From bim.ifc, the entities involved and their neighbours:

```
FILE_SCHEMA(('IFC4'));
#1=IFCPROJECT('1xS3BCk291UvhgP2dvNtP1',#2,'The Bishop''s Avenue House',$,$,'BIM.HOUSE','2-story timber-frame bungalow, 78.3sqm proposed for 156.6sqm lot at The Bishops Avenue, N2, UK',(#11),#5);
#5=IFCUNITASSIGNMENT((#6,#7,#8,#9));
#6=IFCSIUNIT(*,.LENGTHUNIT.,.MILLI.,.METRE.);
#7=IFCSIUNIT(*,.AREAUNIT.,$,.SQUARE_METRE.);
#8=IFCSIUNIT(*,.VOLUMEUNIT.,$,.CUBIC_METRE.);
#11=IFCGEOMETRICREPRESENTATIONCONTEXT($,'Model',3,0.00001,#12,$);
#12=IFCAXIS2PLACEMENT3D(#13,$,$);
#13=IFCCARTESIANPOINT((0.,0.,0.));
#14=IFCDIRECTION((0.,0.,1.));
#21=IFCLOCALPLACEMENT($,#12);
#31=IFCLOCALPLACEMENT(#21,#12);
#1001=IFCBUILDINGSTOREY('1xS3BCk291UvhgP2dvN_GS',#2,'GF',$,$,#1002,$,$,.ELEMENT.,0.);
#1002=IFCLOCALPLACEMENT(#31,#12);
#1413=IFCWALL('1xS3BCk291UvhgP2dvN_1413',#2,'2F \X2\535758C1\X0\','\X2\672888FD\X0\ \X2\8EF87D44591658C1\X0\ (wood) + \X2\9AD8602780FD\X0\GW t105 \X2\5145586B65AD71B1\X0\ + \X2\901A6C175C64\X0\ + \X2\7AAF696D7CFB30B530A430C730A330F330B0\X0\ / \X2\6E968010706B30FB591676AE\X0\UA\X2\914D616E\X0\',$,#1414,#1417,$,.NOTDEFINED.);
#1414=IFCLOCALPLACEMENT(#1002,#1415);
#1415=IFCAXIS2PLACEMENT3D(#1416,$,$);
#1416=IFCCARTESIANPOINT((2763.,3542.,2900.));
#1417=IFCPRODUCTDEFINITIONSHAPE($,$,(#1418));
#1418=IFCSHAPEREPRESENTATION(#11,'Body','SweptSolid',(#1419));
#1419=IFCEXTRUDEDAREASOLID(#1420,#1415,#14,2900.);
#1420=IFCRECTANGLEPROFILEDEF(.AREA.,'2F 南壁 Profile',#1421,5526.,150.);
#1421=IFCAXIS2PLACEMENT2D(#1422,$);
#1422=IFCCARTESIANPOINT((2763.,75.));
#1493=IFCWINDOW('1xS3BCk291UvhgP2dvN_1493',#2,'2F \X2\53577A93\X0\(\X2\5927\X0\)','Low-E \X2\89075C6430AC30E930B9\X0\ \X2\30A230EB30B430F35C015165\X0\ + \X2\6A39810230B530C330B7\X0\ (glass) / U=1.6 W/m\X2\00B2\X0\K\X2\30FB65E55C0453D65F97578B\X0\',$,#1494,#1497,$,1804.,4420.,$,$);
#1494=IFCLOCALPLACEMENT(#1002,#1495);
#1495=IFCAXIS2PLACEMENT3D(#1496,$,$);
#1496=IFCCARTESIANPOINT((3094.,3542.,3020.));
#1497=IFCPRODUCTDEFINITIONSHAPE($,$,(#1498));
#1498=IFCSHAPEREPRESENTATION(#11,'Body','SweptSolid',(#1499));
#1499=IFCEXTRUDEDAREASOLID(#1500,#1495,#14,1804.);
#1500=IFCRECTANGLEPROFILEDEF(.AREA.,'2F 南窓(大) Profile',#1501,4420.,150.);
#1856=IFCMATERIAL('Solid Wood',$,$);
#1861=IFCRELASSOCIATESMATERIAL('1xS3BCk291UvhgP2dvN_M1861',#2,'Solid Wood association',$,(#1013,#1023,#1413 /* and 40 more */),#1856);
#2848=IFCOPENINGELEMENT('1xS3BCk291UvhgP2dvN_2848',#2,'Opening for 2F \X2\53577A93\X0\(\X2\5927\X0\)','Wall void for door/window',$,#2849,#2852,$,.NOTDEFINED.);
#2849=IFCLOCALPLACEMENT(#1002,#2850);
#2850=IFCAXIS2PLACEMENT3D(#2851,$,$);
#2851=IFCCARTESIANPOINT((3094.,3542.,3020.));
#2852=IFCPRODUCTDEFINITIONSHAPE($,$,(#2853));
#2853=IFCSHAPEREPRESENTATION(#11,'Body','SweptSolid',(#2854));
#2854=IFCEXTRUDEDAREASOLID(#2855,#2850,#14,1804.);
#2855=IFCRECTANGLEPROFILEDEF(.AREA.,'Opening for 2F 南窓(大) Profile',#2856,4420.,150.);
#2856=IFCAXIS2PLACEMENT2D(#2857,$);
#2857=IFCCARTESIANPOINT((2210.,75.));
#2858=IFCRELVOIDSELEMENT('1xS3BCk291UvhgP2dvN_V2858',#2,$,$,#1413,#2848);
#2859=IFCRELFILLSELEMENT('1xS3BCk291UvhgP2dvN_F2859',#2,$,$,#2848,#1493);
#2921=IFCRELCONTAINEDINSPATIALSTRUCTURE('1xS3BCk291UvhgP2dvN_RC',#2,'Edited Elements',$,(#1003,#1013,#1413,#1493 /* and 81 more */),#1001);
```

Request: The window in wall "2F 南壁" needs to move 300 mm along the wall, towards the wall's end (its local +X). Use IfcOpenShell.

```python
import ifcopenshell
import ifcopenshell.api.geometry
import ifcopenshell.util.placement
import ifcopenshell.util.unit

model = ifcopenshell.open("bim.ifc")
unit_scale = ifcopenshell.util.unit.calculate_unit_scale(model)

window = model.by_guid("1xS3BCk291UvhgP2dvN_1493")
opening = window.FillsVoids[0].RelatingOpeningElement
wall = opening.VoidsElements[0].RelatingBuildingElement

wall_matrix = ifcopenshell.util.placement.get_local_placement(wall.ObjectPlacement)
shift = wall_matrix[:3, 0] * 0.3 / unit_scale
before = ifcopenshell.util.placement.get_local_placement(window.ObjectPlacement)[:3, 3].copy()

# The window is not placed relative to its opening, so move both.
for product in (opening, window):
    matrix = ifcopenshell.util.placement.get_local_placement(product.ObjectPlacement)
    matrix[:3, 3] += shift
    ifcopenshell.api.geometry.edit_object_placement(model, product=product, matrix=matrix, is_si=False)

after = ifcopenshell.util.placement.get_local_placement(window.ObjectPlacement)[:3, 3]
print("window moved by", (after - before).round(3) + 0.0)

model.write("bim_v2.ifc")
```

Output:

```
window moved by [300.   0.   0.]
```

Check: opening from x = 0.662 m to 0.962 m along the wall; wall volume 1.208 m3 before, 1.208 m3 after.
